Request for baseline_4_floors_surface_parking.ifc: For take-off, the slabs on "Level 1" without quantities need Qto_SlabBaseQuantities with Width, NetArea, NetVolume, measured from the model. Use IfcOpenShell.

First a look at what the model holds.

```python
import ifcopenshell
import ifcopenshell.util.element
import ifcopenshell.util.unit

model = ifcopenshell.open("baseline_4_floors_surface_parking.ifc")
print(model.schema)
for unit_type in ("LENGTHUNIT", "AREAUNIT", "VOLUMEUNIT"):
    print(unit_type, ifcopenshell.util.unit.calculate_unit_scale(model, unit_type))
storey = next(s for s in model.by_type("IfcBuildingStorey") if s.Name == "Level 1")
slabs = [e for e in ifcopenshell.util.element.get_decomposition(storey) if e.is_a("IfcSlab")]
for e in sorted(slabs, key=lambda e: e.id()):
    print(e.id(), e.is_a(), e.Name, list(ifcopenshell.util.element.get_psets(e, qtos_only=True)), sep=" | ")
```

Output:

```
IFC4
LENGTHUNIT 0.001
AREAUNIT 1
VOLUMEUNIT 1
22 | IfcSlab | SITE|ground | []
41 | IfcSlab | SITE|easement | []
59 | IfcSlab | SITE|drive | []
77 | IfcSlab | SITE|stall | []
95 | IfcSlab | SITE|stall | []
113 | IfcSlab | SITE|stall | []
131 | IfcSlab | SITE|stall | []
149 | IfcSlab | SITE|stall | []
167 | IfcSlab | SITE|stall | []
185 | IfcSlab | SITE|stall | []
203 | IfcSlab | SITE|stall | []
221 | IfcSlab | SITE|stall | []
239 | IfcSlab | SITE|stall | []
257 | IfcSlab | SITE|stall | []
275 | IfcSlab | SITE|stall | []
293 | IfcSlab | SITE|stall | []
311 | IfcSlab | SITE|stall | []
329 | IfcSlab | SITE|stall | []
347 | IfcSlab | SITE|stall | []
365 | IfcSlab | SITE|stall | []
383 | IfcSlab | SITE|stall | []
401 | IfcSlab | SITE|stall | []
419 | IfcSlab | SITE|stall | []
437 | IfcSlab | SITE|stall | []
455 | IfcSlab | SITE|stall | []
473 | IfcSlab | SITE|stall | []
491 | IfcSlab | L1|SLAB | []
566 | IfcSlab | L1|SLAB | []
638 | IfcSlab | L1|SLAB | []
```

```python
import ifcopenshell
import ifcopenshell.api.pset
import ifcopenshell.geom
import ifcopenshell.util.element
import ifcopenshell.util.shape
import ifcopenshell.util.unit

model = ifcopenshell.open("baseline_4_floors_surface_parking.ifc")
unit_scale = ifcopenshell.util.unit.calculate_unit_scale(model)
area_scale = ifcopenshell.util.unit.calculate_unit_scale(model, "AREAUNIT")
volume_scale = ifcopenshell.util.unit.calculate_unit_scale(model, "VOLUMEUNIT")
settings = ifcopenshell.geom.settings()

storey = next(s for s in model.by_type("IfcBuildingStorey") if s.Name == "Level 1")
slabs = [e for e in ifcopenshell.util.element.get_decomposition(storey) if e.is_a("IfcSlab")]

for e in sorted(slabs, key=lambda e: e.id()):
    if ifcopenshell.util.element.get_psets(e, qtos_only=True, should_inherit=False):
        continue
    # Geometry comes back in metres, in the element's own axes.
    shape = ifcopenshell.geom.create_shape(settings, e)
    values = {
        "Width": ifcopenshell.util.shape.get_z(shape.geometry) / unit_scale,
        "NetArea": ifcopenshell.util.shape.get_footprint_area(shape.geometry) / area_scale,
        "NetVolume": ifcopenshell.util.shape.get_volume(shape.geometry) / volume_scale,
    }
    qto = ifcopenshell.api.pset.add_qto(model, product=e, name="Qto_SlabBaseQuantities")
    ifcopenshell.api.pset.edit_qto(model, qto=qto, properties=values)
    print(e.id(), {k: round(v, 3) for k, v in values.items()})

model.write("baseline_4_floors_surface_parking-out.ifc")
```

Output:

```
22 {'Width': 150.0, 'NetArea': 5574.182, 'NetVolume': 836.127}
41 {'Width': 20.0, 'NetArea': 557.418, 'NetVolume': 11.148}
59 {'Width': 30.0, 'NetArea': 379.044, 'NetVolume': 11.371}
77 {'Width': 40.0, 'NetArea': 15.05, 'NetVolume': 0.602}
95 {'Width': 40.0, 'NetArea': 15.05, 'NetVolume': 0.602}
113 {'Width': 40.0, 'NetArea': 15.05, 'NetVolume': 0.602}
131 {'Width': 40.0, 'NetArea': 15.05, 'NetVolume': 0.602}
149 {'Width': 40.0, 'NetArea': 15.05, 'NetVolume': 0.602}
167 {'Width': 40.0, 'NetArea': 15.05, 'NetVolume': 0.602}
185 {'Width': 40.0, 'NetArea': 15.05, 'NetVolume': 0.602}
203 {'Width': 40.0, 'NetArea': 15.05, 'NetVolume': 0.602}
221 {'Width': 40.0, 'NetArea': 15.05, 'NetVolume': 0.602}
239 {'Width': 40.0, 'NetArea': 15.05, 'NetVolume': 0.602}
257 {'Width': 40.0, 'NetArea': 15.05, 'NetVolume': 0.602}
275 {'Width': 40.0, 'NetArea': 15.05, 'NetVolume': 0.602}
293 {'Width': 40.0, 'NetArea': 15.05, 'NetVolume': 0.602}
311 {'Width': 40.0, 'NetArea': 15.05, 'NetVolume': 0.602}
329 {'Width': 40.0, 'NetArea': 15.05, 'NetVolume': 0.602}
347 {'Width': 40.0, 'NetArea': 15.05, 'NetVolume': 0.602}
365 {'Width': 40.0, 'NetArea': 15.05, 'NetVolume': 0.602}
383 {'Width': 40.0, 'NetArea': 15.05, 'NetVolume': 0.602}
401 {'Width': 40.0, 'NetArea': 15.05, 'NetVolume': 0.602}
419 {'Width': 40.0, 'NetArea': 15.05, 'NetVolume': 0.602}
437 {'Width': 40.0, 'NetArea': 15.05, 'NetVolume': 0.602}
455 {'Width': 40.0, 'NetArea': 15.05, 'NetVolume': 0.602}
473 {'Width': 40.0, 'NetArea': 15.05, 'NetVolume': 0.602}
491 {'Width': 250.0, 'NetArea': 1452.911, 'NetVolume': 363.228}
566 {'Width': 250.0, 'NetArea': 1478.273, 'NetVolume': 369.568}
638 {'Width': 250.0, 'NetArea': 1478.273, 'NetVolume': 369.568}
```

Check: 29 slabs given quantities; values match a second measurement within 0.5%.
